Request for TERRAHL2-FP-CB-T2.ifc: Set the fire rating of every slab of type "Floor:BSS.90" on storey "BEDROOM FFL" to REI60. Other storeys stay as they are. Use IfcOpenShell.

First a look at what the model holds.

```python
import ifcopenshell
import ifcopenshell.util.element

model = ifcopenshell.open("TERRAHL2-FP-CB-T2.ifc")
print(model.schema)
storey = next(s for s in model.by_type("IfcBuildingStorey") if s.Name == "BEDROOM FFL")
slabs = [e for e in ifcopenshell.util.element.get_decomposition(storey) if e.is_a("IfcSlab")]
seen = {}
for e in slabs:
    element_type = ifcopenshell.util.element.get_type(e)
    key = (element_type.Name if element_type != e and element_type else None, ifcopenshell.util.element.get_pset(e, "Pset_SlabCommon", "FireRating"))
    seen[key] = seen.get(key, 0) + 1
for (name, value), count in sorted(seen.items(), key=str):
    print(count, "x", name, "|", value)
```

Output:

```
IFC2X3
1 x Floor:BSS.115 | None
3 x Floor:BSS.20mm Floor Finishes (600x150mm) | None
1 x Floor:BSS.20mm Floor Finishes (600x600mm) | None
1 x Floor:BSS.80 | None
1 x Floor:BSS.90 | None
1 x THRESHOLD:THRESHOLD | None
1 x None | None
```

```python
import ifcopenshell
import ifcopenshell.api.pset
import ifcopenshell.util.element

model = ifcopenshell.open("TERRAHL2-FP-CB-T2.ifc")

storey = next(s for s in model.by_type("IfcBuildingStorey") if s.Name == "BEDROOM FFL")
slabs = [e for e in ifcopenshell.util.element.get_decomposition(storey) if e.is_a("IfcSlab")]

count = 0
for e in slabs:
    element_type = ifcopenshell.util.element.get_type(e)
    if element_type in (None, e) or element_type.Name != "Floor:BSS.90":
        continue
    # add_pset returns the element's existing set when there is one.
    pset = ifcopenshell.api.pset.add_pset(model, product=e, name="Pset_SlabCommon")
    ifcopenshell.api.pset.edit_pset(model, pset=pset, properties={"FireRating": "REI60"})
    count += 1

print(count, "slabs updated")

model.write("TERRAHL2-FP-CB-T2-out.ifc")
```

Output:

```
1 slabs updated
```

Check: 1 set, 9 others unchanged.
